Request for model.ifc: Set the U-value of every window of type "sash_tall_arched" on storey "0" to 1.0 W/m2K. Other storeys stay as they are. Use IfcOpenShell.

First a look at what the model holds.

```python
import ifcopenshell
import ifcopenshell.util.element

model = ifcopenshell.open("model.ifc")
print(model.schema)
storey = next(s for s in model.by_type("IfcBuildingStorey") if s.Name == "0")
windows = [e for e in ifcopenshell.util.element.get_decomposition(storey) if e.is_a("IfcWindow")]
seen = {}
for e in windows:
    element_type = ifcopenshell.util.element.get_type(e)
    key = (element_type.Name if element_type != e and element_type else None, ifcopenshell.util.element.get_pset(e, "Pset_WindowCommon", "ThermalTransmittance"))
    seen[key] = seen.get(key, 0) + 1
for (name, value), count in sorted(seen.items(), key=str):
    print(count, "x", name, "|", value)
```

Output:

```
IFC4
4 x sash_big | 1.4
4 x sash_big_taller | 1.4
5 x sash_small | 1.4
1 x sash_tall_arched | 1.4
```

```python
import ifcopenshell
import ifcopenshell.api.pset
import ifcopenshell.util.element

model = ifcopenshell.open("model.ifc")

storey = next(s for s in model.by_type("IfcBuildingStorey") if s.Name == "0")
windows = [e for e in ifcopenshell.util.element.get_decomposition(storey) if e.is_a("IfcWindow")]

count = 0
for e in windows:
    element_type = ifcopenshell.util.element.get_type(e)
    if element_type in (None, e) or element_type.Name != "sash_tall_arched":
        continue
    # add_pset returns the element's existing set when there is one.
    pset = ifcopenshell.api.pset.add_pset(model, product=e, name="Pset_WindowCommon")
    ifcopenshell.api.pset.edit_pset(model, pset=pset, properties={"ThermalTransmittance": 1.0})
    count += 1

print(count, "windows updated")

model.write("model-out.ifc")
```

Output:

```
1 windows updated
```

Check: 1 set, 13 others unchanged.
